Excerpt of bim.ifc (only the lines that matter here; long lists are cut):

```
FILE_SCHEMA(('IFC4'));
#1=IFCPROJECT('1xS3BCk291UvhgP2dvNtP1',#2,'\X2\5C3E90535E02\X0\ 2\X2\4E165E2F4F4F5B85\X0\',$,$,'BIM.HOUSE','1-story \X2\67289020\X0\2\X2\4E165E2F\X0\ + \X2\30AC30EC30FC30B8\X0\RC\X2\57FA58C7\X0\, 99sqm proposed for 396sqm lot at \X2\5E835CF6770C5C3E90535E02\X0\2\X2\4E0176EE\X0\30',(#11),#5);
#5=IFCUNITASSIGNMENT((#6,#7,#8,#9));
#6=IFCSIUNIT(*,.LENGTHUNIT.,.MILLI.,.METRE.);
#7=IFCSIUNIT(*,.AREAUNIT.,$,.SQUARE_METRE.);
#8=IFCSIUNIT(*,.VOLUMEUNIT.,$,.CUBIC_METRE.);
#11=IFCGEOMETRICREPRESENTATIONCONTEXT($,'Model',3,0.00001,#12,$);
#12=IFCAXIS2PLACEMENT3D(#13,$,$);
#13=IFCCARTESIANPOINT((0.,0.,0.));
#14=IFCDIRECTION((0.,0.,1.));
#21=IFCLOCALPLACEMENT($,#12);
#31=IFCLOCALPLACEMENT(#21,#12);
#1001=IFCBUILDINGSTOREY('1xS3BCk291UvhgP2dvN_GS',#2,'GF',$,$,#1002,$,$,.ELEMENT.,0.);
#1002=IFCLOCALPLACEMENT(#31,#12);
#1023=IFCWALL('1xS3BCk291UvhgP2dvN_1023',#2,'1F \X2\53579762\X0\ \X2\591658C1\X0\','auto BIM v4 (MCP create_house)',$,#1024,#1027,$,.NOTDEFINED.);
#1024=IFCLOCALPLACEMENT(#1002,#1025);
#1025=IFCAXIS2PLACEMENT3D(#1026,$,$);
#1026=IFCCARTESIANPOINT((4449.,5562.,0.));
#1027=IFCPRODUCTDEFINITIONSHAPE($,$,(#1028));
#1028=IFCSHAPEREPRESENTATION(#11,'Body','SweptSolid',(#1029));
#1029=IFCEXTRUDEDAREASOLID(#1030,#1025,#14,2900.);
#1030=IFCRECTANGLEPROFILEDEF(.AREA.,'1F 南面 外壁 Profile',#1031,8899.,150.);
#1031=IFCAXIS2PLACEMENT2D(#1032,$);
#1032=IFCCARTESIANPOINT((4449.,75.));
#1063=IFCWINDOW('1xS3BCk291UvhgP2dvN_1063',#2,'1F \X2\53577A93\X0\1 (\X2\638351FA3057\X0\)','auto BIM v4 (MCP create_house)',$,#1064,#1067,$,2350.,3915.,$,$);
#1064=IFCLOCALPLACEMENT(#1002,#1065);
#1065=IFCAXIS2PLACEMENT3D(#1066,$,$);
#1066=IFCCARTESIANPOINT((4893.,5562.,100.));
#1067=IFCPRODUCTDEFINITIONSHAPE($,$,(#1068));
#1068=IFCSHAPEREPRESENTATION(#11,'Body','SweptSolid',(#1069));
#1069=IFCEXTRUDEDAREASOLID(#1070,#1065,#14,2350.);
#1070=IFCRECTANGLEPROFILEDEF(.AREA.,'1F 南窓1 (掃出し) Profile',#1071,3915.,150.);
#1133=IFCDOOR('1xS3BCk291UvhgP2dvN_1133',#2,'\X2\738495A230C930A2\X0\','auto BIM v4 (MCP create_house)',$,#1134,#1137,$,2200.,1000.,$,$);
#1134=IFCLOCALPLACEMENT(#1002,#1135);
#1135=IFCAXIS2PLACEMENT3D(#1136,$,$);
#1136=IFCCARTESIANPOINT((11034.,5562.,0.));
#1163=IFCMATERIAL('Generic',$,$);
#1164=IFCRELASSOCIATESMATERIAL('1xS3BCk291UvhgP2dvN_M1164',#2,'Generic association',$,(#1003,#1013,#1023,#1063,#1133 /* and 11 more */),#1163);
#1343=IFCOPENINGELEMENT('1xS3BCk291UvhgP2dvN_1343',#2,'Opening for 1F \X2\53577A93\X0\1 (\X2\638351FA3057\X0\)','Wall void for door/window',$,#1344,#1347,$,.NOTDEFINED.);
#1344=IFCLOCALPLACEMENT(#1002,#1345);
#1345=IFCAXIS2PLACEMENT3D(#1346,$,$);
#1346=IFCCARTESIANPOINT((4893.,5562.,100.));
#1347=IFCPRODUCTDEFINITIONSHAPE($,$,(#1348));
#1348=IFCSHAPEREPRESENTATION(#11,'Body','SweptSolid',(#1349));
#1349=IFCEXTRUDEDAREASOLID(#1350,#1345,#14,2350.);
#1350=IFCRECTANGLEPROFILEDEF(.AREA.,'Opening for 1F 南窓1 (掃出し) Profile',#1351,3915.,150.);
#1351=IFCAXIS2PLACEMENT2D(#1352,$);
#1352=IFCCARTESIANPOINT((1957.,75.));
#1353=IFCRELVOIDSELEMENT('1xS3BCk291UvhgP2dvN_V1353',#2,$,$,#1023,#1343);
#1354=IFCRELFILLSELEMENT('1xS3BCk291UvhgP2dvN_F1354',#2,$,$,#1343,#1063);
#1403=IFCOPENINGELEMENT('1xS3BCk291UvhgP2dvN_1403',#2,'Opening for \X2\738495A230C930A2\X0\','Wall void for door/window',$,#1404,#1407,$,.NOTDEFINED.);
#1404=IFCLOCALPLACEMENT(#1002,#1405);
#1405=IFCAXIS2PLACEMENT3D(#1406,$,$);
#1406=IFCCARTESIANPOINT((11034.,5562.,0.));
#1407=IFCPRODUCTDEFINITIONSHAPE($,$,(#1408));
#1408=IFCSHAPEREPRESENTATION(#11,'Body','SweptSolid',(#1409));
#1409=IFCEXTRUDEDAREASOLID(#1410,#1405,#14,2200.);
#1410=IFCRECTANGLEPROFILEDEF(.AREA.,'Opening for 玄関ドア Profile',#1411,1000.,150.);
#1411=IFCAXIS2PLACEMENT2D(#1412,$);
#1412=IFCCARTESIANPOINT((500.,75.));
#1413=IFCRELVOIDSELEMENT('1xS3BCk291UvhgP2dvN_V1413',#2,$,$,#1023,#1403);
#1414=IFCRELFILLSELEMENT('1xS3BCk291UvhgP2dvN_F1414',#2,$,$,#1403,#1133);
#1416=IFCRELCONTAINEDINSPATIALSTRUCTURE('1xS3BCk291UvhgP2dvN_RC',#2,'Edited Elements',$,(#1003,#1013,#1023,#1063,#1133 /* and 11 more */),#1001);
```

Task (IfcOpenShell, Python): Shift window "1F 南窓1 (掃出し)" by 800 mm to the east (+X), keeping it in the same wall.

```python
import ifcopenshell
import ifcopenshell.api.geometry
import ifcopenshell.util.placement
import ifcopenshell.util.unit

model = ifcopenshell.open("bim.ifc")
unit_scale = ifcopenshell.util.unit.calculate_unit_scale(model)

window = model.by_guid("1xS3BCk291UvhgP2dvN_1063")
opening = window.FillsVoids[0].RelatingOpeningElement
wall = opening.VoidsElements[0].RelatingBuildingElement

wall_matrix = ifcopenshell.util.placement.get_local_placement(wall.ObjectPlacement)
shift = wall_matrix[:3, 0] * 0.8 / unit_scale
before = ifcopenshell.util.placement.get_local_placement(window.ObjectPlacement)[:3, 3].copy()

# The window is not placed relative to its opening, so move both.
for product in (opening, window):
    matrix = ifcopenshell.util.placement.get_local_placement(product.ObjectPlacement)
    matrix[:3, 3] += shift
    ifcopenshell.api.geometry.edit_object_placement(model, product=product, matrix=matrix, is_si=False)

after = ifcopenshell.util.placement.get_local_placement(window.ObjectPlacement)[:3, 3]
print("window moved by", (after - before).round(3) + 0.0)

model.write("bim-out.ifc")
```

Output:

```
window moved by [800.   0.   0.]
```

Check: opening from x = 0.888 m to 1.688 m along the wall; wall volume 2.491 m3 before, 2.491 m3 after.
